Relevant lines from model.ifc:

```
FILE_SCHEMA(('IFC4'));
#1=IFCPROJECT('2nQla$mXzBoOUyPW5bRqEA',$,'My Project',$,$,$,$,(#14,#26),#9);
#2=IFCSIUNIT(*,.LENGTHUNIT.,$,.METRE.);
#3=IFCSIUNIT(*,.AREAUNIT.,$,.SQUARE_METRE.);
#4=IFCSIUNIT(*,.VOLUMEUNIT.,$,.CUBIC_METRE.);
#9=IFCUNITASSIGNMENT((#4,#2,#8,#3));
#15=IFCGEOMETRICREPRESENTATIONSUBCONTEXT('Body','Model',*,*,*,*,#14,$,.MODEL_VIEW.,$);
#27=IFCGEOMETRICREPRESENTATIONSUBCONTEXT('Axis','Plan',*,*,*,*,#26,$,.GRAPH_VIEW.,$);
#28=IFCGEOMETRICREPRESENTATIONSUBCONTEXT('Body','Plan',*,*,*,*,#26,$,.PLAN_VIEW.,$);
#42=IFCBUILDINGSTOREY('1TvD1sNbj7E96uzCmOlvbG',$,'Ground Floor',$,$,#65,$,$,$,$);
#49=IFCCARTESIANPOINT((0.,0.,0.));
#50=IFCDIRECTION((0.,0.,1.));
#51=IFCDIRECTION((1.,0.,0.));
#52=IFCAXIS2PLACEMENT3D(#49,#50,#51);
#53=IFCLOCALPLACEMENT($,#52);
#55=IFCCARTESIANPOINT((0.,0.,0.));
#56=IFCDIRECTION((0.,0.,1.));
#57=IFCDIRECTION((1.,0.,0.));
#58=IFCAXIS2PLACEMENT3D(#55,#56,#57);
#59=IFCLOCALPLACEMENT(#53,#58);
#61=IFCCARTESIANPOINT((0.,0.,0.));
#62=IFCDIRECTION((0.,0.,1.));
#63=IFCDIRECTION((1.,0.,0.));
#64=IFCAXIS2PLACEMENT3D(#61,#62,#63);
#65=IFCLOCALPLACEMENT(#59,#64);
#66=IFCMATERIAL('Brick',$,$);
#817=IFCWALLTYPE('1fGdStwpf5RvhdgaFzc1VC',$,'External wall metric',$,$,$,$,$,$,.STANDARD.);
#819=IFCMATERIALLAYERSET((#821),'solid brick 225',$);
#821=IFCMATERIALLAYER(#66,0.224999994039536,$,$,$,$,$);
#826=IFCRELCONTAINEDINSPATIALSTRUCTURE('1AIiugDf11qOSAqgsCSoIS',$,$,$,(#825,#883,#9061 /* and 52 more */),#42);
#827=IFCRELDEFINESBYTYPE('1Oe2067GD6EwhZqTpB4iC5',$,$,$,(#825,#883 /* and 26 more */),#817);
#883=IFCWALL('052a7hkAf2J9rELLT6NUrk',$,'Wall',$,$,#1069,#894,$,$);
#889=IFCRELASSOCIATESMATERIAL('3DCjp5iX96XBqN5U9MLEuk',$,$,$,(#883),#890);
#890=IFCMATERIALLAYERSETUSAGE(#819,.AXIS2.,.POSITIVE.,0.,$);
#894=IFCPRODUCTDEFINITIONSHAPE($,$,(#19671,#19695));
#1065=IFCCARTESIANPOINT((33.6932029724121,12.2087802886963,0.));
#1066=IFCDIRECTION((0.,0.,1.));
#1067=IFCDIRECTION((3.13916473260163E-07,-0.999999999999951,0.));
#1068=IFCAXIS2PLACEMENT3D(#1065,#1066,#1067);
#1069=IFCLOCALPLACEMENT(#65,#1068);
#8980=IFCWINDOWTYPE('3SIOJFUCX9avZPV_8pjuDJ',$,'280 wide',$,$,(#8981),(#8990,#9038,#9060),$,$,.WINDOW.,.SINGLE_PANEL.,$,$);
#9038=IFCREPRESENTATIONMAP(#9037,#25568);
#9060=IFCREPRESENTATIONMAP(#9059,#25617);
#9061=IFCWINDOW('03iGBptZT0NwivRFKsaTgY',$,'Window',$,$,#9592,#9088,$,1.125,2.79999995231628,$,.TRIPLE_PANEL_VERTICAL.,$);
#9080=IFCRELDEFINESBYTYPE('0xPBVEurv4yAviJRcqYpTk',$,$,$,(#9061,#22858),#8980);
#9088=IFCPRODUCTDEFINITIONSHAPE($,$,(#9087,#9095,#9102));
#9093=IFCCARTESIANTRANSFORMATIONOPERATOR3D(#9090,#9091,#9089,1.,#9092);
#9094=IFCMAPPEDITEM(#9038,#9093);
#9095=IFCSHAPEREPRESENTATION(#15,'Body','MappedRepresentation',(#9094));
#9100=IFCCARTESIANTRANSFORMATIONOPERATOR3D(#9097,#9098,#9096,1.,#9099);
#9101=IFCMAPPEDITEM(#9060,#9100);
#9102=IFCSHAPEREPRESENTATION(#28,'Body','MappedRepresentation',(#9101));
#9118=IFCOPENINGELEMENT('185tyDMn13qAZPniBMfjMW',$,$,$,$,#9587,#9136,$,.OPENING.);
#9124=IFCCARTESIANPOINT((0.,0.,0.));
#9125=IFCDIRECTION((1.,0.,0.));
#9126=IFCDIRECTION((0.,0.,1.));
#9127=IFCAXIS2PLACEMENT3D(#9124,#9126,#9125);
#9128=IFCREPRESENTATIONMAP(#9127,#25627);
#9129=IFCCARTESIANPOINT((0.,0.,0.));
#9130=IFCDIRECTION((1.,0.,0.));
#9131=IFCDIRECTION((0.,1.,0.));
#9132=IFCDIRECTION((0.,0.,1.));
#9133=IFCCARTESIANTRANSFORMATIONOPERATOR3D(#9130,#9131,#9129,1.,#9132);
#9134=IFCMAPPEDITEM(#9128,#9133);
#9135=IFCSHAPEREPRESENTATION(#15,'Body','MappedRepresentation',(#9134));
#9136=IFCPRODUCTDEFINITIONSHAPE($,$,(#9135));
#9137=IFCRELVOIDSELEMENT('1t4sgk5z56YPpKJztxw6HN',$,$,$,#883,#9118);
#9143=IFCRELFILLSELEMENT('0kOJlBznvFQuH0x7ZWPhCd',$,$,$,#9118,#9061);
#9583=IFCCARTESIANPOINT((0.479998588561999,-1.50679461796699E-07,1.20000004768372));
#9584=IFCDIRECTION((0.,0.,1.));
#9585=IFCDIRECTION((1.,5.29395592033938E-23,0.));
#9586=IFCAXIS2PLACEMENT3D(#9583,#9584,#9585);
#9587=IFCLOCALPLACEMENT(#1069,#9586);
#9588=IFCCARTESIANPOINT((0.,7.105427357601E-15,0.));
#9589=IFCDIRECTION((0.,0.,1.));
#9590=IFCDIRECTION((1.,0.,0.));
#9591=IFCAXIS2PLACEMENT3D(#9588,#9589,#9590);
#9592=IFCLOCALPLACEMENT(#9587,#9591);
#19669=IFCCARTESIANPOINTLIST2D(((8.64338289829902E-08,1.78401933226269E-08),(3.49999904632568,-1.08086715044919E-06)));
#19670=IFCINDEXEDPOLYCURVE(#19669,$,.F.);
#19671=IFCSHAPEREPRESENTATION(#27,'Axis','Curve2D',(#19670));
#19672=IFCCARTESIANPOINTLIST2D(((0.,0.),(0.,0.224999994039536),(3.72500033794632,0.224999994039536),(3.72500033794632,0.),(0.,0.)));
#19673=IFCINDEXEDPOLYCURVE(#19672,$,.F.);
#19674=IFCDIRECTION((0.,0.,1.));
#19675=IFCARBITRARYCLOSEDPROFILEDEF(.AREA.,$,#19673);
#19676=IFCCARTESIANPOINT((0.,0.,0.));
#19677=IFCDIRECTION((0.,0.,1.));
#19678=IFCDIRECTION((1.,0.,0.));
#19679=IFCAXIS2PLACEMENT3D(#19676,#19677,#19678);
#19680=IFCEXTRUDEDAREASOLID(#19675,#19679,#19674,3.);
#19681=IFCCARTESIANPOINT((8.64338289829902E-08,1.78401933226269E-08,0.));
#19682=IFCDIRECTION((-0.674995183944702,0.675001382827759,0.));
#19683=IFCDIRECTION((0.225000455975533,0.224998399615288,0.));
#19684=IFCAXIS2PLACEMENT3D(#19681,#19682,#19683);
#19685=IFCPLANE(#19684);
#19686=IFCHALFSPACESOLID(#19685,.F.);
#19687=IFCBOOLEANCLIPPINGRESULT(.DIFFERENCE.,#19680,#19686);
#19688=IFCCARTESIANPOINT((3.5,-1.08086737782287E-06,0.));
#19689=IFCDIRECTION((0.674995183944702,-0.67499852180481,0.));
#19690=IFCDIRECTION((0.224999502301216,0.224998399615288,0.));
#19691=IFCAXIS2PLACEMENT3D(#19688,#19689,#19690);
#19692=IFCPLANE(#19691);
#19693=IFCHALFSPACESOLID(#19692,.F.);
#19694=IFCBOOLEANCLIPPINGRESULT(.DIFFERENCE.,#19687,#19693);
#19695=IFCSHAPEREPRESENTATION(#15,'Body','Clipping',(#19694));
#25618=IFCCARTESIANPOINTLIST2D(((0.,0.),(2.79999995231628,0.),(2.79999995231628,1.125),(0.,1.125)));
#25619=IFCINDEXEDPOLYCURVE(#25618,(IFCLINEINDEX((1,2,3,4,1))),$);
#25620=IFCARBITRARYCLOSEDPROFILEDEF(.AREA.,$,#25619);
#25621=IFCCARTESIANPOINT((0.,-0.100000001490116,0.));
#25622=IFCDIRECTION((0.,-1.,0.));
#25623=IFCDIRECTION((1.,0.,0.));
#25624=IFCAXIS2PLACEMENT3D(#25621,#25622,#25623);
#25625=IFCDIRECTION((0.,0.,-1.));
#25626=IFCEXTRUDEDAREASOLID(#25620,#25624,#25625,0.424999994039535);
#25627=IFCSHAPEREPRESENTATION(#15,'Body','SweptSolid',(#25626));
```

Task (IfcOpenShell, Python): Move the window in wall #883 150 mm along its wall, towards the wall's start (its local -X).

```python
import ifcopenshell
import ifcopenshell.api.geometry
import ifcopenshell.util.placement

model = ifcopenshell.open("model.ifc")

window = model.by_guid("03iGBptZT0NwivRFKsaTgY")
opening = window.FillsVoids[0].RelatingOpeningElement
wall = opening.VoidsElements[0].RelatingBuildingElement

wall_matrix = ifcopenshell.util.placement.get_local_placement(wall.ObjectPlacement)
shift = wall_matrix[:3, 0] * -0.15
before = ifcopenshell.util.placement.get_local_placement(window.ObjectPlacement)[:3, 3].copy()

# The window is placed relative to its opening, so it follows when the opening moves.
matrix = ifcopenshell.util.placement.get_local_placement(opening.ObjectPlacement)
matrix[:3, 3] += shift
ifcopenshell.api.geometry.edit_object_placement(
    model, product=opening, matrix=matrix, is_si=False, should_transform_children=True
)

after = ifcopenshell.util.placement.get_local_placement(window.ObjectPlacement)[:3, 3]
print("window moved by", (after - before).round(3) + 0.0)

model.write("model_v2.ifc")
```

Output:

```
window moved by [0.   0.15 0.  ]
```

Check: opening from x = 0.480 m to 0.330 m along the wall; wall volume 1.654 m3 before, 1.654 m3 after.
